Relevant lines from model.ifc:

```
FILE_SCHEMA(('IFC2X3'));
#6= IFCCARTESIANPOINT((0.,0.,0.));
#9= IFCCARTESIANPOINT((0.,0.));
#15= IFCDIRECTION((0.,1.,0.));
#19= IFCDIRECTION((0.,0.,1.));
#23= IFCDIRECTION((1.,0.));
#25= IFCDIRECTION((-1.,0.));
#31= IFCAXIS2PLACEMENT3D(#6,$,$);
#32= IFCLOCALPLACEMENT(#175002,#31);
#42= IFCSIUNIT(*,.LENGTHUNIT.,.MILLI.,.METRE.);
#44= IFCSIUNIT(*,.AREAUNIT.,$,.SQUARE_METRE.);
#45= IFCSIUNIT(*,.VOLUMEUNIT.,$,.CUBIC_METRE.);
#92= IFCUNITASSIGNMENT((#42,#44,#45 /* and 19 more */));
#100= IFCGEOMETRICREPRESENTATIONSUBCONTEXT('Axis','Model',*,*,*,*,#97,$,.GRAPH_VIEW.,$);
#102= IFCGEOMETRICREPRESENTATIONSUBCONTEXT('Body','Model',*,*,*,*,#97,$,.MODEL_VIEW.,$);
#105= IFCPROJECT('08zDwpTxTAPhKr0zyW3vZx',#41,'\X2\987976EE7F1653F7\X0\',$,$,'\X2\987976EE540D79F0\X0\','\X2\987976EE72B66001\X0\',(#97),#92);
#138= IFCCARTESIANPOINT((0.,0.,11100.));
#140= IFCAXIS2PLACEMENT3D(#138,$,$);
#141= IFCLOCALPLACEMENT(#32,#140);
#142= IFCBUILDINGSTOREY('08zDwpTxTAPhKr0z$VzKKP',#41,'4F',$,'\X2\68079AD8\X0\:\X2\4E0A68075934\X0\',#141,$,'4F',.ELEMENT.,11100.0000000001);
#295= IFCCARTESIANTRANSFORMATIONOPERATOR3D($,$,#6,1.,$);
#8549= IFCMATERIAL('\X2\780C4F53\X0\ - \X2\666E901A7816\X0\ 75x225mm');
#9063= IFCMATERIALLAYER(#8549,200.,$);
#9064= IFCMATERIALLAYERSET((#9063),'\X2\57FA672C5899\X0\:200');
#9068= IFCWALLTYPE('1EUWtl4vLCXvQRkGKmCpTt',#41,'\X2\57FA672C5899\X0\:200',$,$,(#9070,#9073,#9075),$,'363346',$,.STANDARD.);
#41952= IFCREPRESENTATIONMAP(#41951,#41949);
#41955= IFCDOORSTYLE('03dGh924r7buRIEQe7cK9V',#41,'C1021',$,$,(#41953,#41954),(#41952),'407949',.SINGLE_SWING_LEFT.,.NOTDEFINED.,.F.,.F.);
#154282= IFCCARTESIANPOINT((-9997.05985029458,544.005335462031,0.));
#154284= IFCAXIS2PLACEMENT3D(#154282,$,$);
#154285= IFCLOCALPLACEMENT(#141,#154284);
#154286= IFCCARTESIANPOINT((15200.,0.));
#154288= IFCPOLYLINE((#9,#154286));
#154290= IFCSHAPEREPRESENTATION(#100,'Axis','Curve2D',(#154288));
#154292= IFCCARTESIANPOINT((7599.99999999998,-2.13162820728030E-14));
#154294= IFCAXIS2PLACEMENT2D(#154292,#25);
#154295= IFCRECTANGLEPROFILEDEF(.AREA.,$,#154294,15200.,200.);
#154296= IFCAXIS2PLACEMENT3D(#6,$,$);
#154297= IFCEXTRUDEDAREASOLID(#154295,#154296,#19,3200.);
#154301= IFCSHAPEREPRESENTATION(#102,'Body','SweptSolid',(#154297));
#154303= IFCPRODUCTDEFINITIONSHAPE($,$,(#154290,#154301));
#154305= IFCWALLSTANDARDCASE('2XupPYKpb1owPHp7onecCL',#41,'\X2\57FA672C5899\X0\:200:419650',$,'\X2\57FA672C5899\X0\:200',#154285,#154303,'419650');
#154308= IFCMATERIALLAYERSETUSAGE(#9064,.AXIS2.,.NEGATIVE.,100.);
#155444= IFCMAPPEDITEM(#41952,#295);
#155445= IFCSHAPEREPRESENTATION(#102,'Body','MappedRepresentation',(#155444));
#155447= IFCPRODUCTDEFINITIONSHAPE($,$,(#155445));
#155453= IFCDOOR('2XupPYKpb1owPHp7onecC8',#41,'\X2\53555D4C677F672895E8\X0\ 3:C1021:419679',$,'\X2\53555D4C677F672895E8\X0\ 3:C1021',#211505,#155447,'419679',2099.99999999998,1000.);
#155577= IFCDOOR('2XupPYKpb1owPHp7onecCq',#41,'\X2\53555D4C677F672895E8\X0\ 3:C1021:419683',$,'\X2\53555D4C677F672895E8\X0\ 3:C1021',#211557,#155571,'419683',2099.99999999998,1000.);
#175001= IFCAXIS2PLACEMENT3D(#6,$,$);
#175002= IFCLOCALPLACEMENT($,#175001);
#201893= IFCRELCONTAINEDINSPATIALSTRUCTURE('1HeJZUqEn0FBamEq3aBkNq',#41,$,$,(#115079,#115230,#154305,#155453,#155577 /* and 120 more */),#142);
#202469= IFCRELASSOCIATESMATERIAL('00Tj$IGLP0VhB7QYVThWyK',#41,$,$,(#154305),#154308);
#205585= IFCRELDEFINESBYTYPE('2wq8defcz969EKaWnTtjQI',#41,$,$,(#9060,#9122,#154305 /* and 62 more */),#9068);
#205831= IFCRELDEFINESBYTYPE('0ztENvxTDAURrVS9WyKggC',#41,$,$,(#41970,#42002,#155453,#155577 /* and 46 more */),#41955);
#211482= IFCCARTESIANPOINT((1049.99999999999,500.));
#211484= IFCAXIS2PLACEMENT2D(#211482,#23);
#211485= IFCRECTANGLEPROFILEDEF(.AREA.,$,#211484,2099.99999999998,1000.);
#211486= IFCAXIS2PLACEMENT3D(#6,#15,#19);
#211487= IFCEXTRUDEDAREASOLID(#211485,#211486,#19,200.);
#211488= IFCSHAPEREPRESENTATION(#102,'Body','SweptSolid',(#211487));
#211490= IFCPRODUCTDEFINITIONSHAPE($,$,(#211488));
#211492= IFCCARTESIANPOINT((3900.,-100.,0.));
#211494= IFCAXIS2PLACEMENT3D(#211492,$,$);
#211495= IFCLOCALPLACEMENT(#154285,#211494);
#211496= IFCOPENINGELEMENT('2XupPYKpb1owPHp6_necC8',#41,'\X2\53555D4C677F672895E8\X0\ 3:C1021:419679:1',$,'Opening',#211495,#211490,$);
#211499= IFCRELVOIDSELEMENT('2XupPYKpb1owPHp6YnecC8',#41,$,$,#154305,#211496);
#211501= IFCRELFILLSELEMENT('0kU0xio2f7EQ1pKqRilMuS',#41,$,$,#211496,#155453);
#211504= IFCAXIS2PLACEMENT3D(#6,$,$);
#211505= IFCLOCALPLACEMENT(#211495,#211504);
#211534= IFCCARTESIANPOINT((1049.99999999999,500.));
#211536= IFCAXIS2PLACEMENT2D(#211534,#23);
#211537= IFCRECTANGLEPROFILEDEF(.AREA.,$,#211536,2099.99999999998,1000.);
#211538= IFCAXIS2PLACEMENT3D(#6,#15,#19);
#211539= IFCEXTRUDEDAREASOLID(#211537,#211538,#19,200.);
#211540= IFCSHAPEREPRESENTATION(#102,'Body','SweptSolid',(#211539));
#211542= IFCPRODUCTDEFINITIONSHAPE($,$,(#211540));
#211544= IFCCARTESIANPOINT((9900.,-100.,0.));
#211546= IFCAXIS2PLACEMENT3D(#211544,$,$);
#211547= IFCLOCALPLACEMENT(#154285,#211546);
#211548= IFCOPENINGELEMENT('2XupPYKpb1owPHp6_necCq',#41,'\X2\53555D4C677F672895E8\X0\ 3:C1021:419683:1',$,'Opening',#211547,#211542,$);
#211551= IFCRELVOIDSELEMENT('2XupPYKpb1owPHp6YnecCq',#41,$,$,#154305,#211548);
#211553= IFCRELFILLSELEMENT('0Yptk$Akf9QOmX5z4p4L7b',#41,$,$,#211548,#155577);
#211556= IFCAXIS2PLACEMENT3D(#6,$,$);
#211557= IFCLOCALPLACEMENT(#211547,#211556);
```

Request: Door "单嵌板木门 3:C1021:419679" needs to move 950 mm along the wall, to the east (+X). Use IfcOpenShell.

```python
import ifcopenshell
import ifcopenshell.api.geometry
import ifcopenshell.util.placement
import ifcopenshell.util.unit

model = ifcopenshell.open("model.ifc")
unit_scale = ifcopenshell.util.unit.calculate_unit_scale(model)

door = model.by_guid("2XupPYKpb1owPHp7onecC8")
opening = door.FillsVoids[0].RelatingOpeningElement
wall = opening.VoidsElements[0].RelatingBuildingElement

wall_matrix = ifcopenshell.util.placement.get_local_placement(wall.ObjectPlacement)
shift = wall_matrix[:3, 0] * 0.95 / unit_scale
before = ifcopenshell.util.placement.get_local_placement(door.ObjectPlacement)[:3, 3].copy()

# The door is placed relative to its opening, so it follows when the opening moves.
matrix = ifcopenshell.util.placement.get_local_placement(opening.ObjectPlacement)
matrix[:3, 3] += shift
ifcopenshell.api.geometry.edit_object_placement(
    model, product=opening, matrix=matrix, is_si=False, should_transform_children=True
)

after = ifcopenshell.util.placement.get_local_placement(door.ObjectPlacement)[:3, 3]
print("door moved by", (after - before).round(3) + 0.0)

model.write("model_v2.ifc")
```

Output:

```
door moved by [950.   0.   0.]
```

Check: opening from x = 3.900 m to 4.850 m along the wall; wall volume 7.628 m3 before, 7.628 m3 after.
